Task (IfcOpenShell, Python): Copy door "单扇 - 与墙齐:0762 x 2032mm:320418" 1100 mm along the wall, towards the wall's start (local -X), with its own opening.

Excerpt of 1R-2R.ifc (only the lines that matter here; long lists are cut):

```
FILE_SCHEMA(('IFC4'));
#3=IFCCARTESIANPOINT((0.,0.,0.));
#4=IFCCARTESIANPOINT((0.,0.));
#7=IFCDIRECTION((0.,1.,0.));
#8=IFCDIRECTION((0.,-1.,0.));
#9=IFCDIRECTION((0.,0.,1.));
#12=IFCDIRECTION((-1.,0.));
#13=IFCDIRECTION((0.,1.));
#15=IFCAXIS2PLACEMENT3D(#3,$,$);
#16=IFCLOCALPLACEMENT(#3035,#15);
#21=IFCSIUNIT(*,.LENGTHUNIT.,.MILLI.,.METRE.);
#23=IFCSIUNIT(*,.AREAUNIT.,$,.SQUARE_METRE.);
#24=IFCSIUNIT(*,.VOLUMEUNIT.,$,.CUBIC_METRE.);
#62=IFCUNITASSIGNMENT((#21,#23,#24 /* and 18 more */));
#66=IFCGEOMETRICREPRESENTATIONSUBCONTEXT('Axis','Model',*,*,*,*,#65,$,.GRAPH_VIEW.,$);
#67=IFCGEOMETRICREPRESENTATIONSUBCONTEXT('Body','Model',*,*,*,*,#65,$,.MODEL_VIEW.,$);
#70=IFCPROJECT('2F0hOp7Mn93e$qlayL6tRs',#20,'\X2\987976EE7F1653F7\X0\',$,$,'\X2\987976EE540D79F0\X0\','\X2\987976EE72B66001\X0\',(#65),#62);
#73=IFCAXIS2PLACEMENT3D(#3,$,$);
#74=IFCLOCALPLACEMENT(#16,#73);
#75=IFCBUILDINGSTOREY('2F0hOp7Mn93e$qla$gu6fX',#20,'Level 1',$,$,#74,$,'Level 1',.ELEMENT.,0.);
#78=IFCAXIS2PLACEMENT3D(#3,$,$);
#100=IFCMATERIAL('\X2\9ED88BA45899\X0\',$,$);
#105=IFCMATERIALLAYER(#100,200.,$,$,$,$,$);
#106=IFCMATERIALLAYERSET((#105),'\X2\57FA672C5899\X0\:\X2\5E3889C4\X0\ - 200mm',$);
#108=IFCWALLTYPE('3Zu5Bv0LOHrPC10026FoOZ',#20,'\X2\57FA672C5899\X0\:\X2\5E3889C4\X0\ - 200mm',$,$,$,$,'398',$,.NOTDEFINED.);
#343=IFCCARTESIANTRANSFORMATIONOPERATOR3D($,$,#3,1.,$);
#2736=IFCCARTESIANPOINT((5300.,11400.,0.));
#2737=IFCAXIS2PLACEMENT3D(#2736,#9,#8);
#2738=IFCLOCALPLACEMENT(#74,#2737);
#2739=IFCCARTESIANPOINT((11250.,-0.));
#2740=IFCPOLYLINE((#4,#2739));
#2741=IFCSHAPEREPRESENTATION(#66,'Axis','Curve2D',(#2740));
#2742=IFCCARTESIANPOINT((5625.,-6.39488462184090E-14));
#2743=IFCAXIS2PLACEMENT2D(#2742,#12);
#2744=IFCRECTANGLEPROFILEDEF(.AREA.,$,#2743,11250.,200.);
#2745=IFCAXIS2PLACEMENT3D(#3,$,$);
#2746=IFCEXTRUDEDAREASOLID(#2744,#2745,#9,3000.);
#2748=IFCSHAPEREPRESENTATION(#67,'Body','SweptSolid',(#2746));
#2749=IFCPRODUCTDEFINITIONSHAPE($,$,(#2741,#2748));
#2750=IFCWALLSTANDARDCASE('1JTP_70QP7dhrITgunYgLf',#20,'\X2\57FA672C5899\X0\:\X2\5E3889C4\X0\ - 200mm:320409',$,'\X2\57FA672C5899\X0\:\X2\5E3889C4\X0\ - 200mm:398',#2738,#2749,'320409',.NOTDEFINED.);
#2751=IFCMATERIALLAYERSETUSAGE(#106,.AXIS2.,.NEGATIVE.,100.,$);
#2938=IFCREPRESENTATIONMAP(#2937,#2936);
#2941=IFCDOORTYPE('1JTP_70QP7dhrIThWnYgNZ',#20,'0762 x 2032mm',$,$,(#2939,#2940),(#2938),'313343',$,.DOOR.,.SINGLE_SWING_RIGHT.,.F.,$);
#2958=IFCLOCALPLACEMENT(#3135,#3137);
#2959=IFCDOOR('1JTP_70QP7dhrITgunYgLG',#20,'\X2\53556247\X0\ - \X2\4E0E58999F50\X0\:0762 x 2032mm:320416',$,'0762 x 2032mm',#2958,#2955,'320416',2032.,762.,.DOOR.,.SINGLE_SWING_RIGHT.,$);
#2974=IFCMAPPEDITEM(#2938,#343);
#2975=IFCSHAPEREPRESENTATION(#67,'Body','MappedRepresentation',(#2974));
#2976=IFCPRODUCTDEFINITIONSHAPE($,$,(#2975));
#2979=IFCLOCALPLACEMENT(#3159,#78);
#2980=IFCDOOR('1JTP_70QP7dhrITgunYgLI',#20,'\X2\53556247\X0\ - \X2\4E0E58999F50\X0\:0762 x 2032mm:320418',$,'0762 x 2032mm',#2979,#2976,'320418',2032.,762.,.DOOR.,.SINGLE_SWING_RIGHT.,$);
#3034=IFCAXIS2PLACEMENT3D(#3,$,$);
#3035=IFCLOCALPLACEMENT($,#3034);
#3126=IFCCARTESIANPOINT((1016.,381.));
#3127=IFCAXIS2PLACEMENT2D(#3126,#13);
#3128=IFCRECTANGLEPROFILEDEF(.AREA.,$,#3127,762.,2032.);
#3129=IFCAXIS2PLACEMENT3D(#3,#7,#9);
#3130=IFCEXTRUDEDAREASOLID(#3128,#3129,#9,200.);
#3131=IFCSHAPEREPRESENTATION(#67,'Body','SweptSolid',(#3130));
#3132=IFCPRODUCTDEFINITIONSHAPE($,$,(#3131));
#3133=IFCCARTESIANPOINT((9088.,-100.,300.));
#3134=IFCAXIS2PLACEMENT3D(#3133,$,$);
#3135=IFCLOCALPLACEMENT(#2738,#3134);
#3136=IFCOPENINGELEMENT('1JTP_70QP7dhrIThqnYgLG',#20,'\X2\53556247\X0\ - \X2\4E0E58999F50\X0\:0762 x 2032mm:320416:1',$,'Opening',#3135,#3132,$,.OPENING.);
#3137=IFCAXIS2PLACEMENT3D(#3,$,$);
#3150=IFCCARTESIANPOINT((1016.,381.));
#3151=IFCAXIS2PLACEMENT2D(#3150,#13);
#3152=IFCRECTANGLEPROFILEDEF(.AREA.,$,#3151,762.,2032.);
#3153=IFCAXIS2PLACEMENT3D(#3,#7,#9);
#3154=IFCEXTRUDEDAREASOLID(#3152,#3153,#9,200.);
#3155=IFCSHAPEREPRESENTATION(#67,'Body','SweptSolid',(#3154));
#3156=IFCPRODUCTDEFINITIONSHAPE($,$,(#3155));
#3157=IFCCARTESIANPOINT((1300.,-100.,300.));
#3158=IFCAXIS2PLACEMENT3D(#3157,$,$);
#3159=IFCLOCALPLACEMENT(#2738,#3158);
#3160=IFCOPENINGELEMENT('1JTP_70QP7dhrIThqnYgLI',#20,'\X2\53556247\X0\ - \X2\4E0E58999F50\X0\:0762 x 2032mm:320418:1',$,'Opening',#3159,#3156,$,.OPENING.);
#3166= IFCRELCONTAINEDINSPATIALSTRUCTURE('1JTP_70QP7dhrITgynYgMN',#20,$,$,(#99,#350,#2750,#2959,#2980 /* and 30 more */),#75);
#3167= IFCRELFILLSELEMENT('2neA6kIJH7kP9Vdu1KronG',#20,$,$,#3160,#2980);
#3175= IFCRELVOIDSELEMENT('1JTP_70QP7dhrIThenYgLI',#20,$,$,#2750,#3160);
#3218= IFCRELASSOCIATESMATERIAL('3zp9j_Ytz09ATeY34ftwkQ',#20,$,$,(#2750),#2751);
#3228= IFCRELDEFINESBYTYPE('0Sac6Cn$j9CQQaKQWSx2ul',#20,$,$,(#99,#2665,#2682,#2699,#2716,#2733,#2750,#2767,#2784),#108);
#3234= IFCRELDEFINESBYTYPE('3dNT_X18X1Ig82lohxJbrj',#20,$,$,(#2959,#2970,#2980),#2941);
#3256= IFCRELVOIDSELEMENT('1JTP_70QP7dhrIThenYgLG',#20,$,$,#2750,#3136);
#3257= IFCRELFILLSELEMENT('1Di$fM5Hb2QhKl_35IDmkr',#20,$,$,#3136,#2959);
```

```python
import ifcopenshell
import ifcopenshell.api.feature
import ifcopenshell.api.geometry
import ifcopenshell.api.root
import ifcopenshell.geom
import ifcopenshell.util.element
import ifcopenshell.util.placement
import ifcopenshell.util.shape
import ifcopenshell.util.unit

model = ifcopenshell.open("1R-2R.ifc")
unit_scale = ifcopenshell.util.unit.calculate_unit_scale(model)
settings = ifcopenshell.geom.settings()


def volume(element):
    """Net volume in cubic metres, openings subtracted."""
    shape = ifcopenshell.geom.create_shape(settings, element)
    return ifcopenshell.util.shape.get_volume(shape.geometry)


def reuse_history(source, copy):
    """copy_class also copies each property set's owner history, people and application; keep the originals."""
    for rel in copy.IsDefinedBy:
        if rel.is_a("IfcRelDefinesByProperties") and (history := rel.RelatingPropertyDefinition.OwnerHistory):
            rel.RelatingPropertyDefinition.OwnerHistory = source.OwnerHistory
            ifcopenshell.util.element.remove_deep2(model, history)


door = model.by_guid("1JTP_70QP7dhrITgunYgLI")
opening = door.FillsVoids[0].RelatingOpeningElement
wall = opening.VoidsElements[0].RelatingBuildingElement
before = volume(wall)
shift = ifcopenshell.util.placement.get_local_placement(wall.ObjectPlacement)[:3, 0] * -1.1 / unit_scale

# copy_class copies the void relationship, type, container and properties, but no geometry.
new_opening = ifcopenshell.api.root.copy_class(model, product=opening)
new_opening.Representation = ifcopenshell.util.element.copy_deep(
    model, opening.Representation, exclude=["IfcGeometricRepresentationContext", "IfcRepresentationMap"]
)
new_opening.Name = "单扇 - 与墙齐:0762 x 2032mm"
new_door = ifcopenshell.api.root.copy_class(model, product=door)
new_door.Representation = ifcopenshell.util.element.copy_deep(
    model, door.Representation, exclude=["IfcGeometricRepresentationContext", "IfcRepresentationMap"]
)
new_door.Name = "单扇 - 与墙齐:0762 x 2032mm"
new_door.Tag = None
reuse_history(door, new_door)
ifcopenshell.api.feature.add_filling(model, opening=new_opening, element=new_door)

for old, new in ((opening, new_opening), (door, new_door)):
    matrix = ifcopenshell.util.placement.get_local_placement(old.ObjectPlacement)
    matrix[:3, 3] += shift
    ifcopenshell.api.geometry.edit_object_placement(model, product=new, matrix=matrix, is_si=False)

after = volume(wall)

print(f"wall volume {before:.3f} -> {after:.3f} m3")

model.write("1R-2R_rev.ifc")
```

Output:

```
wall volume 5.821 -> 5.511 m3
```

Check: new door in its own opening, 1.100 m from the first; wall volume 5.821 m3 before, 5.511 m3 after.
